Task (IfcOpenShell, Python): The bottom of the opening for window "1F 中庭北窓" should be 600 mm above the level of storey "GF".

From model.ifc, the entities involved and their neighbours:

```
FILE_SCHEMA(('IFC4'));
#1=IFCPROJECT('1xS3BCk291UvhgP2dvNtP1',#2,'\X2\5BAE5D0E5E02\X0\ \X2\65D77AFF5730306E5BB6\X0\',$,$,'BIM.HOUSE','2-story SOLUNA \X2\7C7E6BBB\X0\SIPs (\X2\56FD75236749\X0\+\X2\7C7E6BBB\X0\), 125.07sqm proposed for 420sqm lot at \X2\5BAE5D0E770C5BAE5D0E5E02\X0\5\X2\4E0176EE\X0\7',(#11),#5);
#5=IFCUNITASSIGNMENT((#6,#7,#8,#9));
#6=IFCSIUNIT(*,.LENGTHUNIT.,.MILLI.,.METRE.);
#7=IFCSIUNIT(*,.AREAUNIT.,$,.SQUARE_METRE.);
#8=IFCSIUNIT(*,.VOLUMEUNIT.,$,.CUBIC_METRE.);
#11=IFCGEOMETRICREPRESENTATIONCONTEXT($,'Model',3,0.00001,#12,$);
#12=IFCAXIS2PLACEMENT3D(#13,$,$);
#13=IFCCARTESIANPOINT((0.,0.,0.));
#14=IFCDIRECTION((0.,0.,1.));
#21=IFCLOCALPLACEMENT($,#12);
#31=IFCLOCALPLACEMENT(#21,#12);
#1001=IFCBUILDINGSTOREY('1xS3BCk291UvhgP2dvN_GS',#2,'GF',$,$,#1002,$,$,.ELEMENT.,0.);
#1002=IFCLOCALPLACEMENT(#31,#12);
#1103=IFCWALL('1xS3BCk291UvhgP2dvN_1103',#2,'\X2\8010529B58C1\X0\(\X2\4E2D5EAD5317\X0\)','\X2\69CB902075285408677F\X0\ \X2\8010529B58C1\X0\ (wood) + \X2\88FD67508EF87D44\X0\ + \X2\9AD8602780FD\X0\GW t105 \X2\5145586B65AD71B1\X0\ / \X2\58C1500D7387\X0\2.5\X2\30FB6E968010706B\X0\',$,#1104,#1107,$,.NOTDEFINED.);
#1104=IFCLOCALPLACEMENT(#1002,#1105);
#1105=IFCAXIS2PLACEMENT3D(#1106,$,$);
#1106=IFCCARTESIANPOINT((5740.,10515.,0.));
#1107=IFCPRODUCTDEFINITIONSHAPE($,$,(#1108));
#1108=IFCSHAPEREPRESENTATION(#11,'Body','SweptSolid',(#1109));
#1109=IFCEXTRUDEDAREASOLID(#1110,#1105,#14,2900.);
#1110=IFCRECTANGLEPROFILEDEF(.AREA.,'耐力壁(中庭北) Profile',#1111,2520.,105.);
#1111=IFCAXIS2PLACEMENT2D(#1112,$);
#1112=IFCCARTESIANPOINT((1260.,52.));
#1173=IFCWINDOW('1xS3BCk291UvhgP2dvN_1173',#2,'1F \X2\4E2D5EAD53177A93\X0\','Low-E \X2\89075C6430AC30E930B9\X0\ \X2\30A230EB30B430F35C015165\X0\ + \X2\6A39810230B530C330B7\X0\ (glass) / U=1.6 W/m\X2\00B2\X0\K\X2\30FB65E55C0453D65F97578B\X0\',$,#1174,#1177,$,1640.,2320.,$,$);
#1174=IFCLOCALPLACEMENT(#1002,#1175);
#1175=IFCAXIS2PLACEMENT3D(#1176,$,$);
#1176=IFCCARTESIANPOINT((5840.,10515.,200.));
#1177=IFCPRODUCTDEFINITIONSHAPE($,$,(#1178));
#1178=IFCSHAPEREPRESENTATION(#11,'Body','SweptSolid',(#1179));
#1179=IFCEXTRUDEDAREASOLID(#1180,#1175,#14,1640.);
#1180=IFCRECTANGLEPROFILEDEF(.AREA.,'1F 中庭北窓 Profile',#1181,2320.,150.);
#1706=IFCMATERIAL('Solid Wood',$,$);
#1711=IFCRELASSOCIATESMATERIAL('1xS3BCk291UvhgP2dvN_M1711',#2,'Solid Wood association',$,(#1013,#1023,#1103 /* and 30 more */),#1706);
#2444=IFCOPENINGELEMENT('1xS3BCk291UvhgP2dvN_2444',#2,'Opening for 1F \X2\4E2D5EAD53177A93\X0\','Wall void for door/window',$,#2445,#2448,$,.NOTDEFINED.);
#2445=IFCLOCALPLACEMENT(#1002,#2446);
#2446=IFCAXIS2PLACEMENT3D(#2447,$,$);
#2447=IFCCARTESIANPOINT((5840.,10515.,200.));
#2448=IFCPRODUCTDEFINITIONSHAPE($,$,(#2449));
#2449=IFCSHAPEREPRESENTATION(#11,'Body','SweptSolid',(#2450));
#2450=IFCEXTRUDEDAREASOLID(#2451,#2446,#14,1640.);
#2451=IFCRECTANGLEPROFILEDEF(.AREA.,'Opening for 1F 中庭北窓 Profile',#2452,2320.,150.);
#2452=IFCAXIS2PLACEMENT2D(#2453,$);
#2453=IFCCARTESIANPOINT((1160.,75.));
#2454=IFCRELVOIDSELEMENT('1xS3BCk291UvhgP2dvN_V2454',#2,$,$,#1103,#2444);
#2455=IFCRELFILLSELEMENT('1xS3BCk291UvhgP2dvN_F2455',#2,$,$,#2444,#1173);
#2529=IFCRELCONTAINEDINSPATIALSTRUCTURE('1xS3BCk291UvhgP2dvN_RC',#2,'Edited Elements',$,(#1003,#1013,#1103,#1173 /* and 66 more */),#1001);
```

```python
import numpy as np
import ifcopenshell
import ifcopenshell.api.geometry
import ifcopenshell.geom
import ifcopenshell.util.element
import ifcopenshell.util.placement
import ifcopenshell.util.shape
import ifcopenshell.util.unit

model = ifcopenshell.open("model.ifc")
unit_scale = ifcopenshell.util.unit.calculate_unit_scale(model)

window = model.by_guid("1xS3BCk291UvhgP2dvN_1173")
opening = window.FillsVoids[0].RelatingOpeningElement
storey = ifcopenshell.util.element.get_container(window, ifc_class="IfcBuildingStorey")
level = ifcopenshell.util.placement.get_local_placement(storey.ObjectPlacement)[2, 3]

# The opening's origin need not be at the sill, so measure its lowest point.
shape = ifcopenshell.geom.create_shape(ifcopenshell.geom.settings(), opening)
bottom = ifcopenshell.util.shape.get_shape_bottom_elevation(shape, shape.geometry) / unit_scale
dz = level + 0.6 / unit_scale - bottom

shift = np.array([0.0, 0.0, dz])
# The window is not placed relative to its opening, so move both.
for product in (opening, window):
    matrix = ifcopenshell.util.placement.get_local_placement(product.ObjectPlacement)
    matrix[:3, 3] += shift
    ifcopenshell.api.geometry.edit_object_placement(model, product=product, matrix=matrix, is_si=False)

print(f"moved by {dz * unit_scale:+.3f} m")

model.write("model_v2.ifc")
```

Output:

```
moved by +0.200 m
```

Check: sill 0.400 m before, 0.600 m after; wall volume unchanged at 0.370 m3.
